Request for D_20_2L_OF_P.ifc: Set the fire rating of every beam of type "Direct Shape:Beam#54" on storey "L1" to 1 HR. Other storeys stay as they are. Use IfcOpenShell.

First a look at what the model holds.

```python
import ifcopenshell
import ifcopenshell.util.element

model = ifcopenshell.open("D_20_2L_OF_P.ifc")
print(model.schema)
storey = next(s for s in model.by_type("IfcBuildingStorey") if s.Name == "L1")
beams = [e for e in ifcopenshell.util.element.get_decomposition(storey) if e.is_a("IfcBeam")]
seen = {}
for e in beams:
    element_type = ifcopenshell.util.element.get_type(e)
    key = (element_type.Name if element_type != e and element_type else None, ifcopenshell.util.element.get_pset(e, "Pset_BeamCommon", "FireRating"))
    seen[key] = seen.get(key, 0) + 1
for (name, value), count in sorted(seen.items(), key=str):
    print(count, "x", name, "|", value)
```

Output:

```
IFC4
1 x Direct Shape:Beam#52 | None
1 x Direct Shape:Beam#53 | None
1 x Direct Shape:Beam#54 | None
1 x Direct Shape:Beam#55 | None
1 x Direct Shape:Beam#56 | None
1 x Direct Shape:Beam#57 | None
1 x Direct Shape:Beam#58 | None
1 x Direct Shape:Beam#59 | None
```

```python
import ifcopenshell
import ifcopenshell.api.pset
import ifcopenshell.util.element

model = ifcopenshell.open("D_20_2L_OF_P.ifc")

storey = next(s for s in model.by_type("IfcBuildingStorey") if s.Name == "L1")
beams = [e for e in ifcopenshell.util.element.get_decomposition(storey) if e.is_a("IfcBeam")]

count = 0
for e in beams:
    element_type = ifcopenshell.util.element.get_type(e)
    if element_type in (None, e) or element_type.Name != "Direct Shape:Beam#54":
        continue
    # add_pset returns the element's existing set when there is one.
    pset = ifcopenshell.api.pset.add_pset(model, product=e, name="Pset_BeamCommon")
    ifcopenshell.api.pset.edit_pset(model, pset=pset, properties={"FireRating": "1 HR"})
    count += 1

print(count, "beams updated")

model.write("D_20_2L_OF_P_edited.ifc")
```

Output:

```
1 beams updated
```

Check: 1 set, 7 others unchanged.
